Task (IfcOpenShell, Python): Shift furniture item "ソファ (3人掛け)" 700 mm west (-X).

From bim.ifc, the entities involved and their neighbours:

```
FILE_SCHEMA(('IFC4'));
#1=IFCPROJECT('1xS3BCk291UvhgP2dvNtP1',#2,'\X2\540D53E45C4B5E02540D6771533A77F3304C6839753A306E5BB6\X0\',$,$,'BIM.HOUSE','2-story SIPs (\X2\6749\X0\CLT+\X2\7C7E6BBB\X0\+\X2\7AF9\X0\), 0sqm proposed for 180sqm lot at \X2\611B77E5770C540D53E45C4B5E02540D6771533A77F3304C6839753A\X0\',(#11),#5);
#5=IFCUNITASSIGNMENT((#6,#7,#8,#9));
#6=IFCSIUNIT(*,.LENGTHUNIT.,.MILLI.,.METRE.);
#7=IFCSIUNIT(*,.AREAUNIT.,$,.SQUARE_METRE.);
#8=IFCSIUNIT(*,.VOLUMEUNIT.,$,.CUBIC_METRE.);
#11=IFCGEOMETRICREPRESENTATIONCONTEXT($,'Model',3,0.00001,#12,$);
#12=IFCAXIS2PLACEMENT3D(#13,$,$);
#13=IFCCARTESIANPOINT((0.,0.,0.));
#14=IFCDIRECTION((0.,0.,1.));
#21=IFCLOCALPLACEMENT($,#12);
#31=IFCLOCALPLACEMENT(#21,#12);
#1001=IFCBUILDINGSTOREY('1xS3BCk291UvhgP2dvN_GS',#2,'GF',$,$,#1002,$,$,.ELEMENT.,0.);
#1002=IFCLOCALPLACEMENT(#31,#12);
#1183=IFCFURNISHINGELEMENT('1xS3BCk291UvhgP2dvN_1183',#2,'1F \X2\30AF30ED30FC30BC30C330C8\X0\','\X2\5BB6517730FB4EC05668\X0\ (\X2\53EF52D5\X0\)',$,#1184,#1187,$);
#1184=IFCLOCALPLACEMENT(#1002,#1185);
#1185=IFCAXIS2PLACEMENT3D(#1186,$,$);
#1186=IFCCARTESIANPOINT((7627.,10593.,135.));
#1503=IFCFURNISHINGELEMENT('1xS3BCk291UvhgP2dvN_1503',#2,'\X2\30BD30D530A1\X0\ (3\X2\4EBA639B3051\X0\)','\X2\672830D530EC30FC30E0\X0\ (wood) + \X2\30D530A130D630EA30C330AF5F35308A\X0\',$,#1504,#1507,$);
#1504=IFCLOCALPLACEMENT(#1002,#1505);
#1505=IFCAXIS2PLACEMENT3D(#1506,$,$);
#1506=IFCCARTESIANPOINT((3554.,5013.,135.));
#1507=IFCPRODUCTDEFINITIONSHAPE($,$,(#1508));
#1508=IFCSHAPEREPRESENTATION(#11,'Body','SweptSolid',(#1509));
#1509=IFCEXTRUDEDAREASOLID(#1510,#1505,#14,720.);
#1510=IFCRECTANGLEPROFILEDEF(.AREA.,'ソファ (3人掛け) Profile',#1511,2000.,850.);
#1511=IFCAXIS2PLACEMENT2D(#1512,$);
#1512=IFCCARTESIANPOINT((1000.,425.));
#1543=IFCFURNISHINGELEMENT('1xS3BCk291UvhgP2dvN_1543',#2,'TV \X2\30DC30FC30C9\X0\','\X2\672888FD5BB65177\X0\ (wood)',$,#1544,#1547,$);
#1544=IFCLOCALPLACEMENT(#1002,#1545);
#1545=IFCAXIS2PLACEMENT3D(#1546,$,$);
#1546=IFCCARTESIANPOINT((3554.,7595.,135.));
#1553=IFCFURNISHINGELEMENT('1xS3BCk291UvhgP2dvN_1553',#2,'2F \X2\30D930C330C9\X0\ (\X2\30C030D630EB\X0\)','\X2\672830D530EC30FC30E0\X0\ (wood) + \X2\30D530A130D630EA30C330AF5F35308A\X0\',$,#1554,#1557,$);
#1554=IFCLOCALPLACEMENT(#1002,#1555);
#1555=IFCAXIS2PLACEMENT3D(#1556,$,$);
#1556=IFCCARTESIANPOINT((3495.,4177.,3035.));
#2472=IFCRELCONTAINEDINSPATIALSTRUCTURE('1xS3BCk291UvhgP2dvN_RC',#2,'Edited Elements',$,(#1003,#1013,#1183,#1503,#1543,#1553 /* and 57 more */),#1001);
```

```python
import ifcopenshell
import ifcopenshell.api.geometry
import ifcopenshell.util.placement
import ifcopenshell.util.unit

model = ifcopenshell.open("bim.ifc")
unit_scale = ifcopenshell.util.unit.calculate_unit_scale(model)

item = model.by_id(1503)
matrix = ifcopenshell.util.placement.get_local_placement(item.ObjectPlacement)
matrix[0, 3] -= 0.7 / unit_scale
ifcopenshell.api.geometry.edit_object_placement(model, product=item, matrix=matrix, is_si=False)

print(ifcopenshell.util.placement.get_local_placement(item.ObjectPlacement).round(3) + 0.0)

model.write("bim-out.ifc")
```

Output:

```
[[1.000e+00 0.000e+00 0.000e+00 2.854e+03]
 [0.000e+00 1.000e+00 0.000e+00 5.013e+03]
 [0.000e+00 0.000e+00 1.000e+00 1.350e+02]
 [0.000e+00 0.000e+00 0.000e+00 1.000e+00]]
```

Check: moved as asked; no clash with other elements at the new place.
